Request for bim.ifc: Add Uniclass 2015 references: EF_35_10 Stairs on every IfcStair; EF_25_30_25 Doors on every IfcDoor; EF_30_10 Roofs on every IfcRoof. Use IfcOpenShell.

First a look at what the model holds.

```python
import ifcopenshell

model = ifcopenshell.open("bim.ifc")
print(model.schema)
print("classifications:", [c.Name for c in model.by_type("IfcClassification")])
for ifc_class in ("IfcDoor", "IfcRoof", "IfcStair", "IfcWall", "IfcWindow"):
    print(ifc_class, len(model.by_type(ifc_class)))
```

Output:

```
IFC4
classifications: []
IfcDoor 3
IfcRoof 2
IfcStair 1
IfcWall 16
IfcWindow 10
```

```python
import ifcopenshell
import ifcopenshell.api.classification

model = ifcopenshell.open("bim.ifc")

system = ifcopenshell.api.classification.add_classification(model, classification="Uniclass 2015")

codes = {
    "IfcStair": ("EF_35_10", "Stairs"),
    "IfcDoor": ("EF_25_30_25", "Doors"),
    "IfcRoof": ("EF_30_10", "Roofs"),
}
for ifc_class, (code, name) in codes.items():
    products = model.by_type(ifc_class)
    ifcopenshell.api.classification.add_reference(
        model, products=products, classification=system, identification=code, name=name
    )
    print(code, len(products))

model.write("bim_v2.ifc")
```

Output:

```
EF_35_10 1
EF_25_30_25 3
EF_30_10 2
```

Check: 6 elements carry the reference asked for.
